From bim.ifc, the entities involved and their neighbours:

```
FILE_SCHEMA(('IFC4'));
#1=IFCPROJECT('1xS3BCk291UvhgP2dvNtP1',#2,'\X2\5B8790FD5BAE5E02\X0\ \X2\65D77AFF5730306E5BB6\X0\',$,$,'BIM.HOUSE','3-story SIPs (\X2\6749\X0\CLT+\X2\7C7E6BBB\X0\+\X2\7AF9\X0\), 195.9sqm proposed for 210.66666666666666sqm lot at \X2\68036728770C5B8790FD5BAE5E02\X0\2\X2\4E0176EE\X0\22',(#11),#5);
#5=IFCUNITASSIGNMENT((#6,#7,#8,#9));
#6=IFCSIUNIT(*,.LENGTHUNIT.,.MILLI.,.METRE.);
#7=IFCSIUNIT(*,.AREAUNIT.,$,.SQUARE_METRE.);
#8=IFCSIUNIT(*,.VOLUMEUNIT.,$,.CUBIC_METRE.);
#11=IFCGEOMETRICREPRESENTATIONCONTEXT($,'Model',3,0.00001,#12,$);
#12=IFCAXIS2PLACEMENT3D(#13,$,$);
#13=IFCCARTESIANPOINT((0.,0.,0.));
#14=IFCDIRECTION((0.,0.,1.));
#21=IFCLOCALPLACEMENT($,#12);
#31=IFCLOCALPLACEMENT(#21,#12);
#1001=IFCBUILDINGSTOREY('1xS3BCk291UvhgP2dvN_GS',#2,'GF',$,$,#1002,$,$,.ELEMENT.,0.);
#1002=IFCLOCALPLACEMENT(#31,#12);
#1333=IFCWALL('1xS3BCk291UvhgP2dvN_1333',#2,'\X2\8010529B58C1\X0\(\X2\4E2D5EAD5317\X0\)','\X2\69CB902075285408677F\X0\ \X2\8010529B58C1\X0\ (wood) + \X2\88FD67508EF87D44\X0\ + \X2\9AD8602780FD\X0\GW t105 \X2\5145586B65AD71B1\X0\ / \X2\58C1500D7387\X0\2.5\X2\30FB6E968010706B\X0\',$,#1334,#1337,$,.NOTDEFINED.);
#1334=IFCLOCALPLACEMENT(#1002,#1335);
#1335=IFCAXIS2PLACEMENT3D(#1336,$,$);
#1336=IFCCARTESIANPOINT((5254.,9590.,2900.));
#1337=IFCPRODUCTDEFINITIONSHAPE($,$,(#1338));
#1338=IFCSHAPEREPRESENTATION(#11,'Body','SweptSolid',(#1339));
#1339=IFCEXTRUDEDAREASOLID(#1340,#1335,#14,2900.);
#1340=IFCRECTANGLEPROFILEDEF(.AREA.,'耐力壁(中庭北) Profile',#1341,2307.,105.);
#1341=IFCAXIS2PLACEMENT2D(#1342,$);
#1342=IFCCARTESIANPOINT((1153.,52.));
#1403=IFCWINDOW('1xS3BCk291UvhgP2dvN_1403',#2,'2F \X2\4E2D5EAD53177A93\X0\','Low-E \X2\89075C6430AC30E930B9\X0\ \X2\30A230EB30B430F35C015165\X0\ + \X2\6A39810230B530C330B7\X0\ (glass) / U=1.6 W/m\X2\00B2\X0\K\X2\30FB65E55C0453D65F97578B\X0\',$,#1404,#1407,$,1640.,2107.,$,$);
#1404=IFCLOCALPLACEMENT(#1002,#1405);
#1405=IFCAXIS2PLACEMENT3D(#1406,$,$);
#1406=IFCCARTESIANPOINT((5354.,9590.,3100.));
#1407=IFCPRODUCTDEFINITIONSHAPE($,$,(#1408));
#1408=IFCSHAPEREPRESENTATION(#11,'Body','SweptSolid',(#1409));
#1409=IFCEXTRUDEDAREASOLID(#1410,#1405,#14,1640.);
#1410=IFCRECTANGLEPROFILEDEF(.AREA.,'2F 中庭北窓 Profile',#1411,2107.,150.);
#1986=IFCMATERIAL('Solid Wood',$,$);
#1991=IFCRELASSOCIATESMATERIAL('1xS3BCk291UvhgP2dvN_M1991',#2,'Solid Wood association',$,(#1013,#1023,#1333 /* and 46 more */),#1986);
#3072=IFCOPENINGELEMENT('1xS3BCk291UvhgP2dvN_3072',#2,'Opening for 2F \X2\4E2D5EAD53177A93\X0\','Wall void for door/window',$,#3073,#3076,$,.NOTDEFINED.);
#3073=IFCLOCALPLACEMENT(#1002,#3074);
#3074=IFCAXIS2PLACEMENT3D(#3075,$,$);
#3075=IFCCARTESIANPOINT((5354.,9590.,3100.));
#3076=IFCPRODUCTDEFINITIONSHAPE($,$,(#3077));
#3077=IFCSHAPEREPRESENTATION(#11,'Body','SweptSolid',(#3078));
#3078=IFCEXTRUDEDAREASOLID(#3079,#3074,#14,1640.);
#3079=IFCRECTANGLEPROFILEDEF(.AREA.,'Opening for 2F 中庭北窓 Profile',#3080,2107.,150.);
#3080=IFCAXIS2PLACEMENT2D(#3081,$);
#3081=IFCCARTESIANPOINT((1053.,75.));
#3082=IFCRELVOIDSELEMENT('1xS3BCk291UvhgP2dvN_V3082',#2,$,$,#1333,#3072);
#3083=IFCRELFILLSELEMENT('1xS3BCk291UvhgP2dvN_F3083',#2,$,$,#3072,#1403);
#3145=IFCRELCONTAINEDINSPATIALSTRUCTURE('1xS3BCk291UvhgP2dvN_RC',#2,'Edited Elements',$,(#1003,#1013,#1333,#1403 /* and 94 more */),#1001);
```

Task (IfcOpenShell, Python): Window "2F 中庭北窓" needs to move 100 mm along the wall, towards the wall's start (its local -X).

```python
import ifcopenshell
import ifcopenshell.api.geometry
import ifcopenshell.util.placement

model = ifcopenshell.open("bim.ifc")

window = model.by_guid("1xS3BCk291UvhgP2dvN_1403")
opening = window.FillsVoids[0].RelatingOpeningElement
wall = opening.VoidsElements[0].RelatingBuildingElement

wall_matrix = ifcopenshell.util.placement.get_local_placement(wall.ObjectPlacement)
shift = wall_matrix[:3, 0] * -100.0
before = ifcopenshell.util.placement.get_local_placement(window.ObjectPlacement)[:3, 3].copy()

# The window is not placed relative to its opening, so move both.
for product in (opening, window):
    matrix = ifcopenshell.util.placement.get_local_placement(product.ObjectPlacement)
    matrix[:3, 3] += shift
    ifcopenshell.api.geometry.edit_object_placement(model, product=product, matrix=matrix, is_si=False)

after = ifcopenshell.util.placement.get_local_placement(window.ObjectPlacement)[:3, 3]
print("window moved by", (after - before).round(3) + 0.0)

model.write("bim-out.ifc")
```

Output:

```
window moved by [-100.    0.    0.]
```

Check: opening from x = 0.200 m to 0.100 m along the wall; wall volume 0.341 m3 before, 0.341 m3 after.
